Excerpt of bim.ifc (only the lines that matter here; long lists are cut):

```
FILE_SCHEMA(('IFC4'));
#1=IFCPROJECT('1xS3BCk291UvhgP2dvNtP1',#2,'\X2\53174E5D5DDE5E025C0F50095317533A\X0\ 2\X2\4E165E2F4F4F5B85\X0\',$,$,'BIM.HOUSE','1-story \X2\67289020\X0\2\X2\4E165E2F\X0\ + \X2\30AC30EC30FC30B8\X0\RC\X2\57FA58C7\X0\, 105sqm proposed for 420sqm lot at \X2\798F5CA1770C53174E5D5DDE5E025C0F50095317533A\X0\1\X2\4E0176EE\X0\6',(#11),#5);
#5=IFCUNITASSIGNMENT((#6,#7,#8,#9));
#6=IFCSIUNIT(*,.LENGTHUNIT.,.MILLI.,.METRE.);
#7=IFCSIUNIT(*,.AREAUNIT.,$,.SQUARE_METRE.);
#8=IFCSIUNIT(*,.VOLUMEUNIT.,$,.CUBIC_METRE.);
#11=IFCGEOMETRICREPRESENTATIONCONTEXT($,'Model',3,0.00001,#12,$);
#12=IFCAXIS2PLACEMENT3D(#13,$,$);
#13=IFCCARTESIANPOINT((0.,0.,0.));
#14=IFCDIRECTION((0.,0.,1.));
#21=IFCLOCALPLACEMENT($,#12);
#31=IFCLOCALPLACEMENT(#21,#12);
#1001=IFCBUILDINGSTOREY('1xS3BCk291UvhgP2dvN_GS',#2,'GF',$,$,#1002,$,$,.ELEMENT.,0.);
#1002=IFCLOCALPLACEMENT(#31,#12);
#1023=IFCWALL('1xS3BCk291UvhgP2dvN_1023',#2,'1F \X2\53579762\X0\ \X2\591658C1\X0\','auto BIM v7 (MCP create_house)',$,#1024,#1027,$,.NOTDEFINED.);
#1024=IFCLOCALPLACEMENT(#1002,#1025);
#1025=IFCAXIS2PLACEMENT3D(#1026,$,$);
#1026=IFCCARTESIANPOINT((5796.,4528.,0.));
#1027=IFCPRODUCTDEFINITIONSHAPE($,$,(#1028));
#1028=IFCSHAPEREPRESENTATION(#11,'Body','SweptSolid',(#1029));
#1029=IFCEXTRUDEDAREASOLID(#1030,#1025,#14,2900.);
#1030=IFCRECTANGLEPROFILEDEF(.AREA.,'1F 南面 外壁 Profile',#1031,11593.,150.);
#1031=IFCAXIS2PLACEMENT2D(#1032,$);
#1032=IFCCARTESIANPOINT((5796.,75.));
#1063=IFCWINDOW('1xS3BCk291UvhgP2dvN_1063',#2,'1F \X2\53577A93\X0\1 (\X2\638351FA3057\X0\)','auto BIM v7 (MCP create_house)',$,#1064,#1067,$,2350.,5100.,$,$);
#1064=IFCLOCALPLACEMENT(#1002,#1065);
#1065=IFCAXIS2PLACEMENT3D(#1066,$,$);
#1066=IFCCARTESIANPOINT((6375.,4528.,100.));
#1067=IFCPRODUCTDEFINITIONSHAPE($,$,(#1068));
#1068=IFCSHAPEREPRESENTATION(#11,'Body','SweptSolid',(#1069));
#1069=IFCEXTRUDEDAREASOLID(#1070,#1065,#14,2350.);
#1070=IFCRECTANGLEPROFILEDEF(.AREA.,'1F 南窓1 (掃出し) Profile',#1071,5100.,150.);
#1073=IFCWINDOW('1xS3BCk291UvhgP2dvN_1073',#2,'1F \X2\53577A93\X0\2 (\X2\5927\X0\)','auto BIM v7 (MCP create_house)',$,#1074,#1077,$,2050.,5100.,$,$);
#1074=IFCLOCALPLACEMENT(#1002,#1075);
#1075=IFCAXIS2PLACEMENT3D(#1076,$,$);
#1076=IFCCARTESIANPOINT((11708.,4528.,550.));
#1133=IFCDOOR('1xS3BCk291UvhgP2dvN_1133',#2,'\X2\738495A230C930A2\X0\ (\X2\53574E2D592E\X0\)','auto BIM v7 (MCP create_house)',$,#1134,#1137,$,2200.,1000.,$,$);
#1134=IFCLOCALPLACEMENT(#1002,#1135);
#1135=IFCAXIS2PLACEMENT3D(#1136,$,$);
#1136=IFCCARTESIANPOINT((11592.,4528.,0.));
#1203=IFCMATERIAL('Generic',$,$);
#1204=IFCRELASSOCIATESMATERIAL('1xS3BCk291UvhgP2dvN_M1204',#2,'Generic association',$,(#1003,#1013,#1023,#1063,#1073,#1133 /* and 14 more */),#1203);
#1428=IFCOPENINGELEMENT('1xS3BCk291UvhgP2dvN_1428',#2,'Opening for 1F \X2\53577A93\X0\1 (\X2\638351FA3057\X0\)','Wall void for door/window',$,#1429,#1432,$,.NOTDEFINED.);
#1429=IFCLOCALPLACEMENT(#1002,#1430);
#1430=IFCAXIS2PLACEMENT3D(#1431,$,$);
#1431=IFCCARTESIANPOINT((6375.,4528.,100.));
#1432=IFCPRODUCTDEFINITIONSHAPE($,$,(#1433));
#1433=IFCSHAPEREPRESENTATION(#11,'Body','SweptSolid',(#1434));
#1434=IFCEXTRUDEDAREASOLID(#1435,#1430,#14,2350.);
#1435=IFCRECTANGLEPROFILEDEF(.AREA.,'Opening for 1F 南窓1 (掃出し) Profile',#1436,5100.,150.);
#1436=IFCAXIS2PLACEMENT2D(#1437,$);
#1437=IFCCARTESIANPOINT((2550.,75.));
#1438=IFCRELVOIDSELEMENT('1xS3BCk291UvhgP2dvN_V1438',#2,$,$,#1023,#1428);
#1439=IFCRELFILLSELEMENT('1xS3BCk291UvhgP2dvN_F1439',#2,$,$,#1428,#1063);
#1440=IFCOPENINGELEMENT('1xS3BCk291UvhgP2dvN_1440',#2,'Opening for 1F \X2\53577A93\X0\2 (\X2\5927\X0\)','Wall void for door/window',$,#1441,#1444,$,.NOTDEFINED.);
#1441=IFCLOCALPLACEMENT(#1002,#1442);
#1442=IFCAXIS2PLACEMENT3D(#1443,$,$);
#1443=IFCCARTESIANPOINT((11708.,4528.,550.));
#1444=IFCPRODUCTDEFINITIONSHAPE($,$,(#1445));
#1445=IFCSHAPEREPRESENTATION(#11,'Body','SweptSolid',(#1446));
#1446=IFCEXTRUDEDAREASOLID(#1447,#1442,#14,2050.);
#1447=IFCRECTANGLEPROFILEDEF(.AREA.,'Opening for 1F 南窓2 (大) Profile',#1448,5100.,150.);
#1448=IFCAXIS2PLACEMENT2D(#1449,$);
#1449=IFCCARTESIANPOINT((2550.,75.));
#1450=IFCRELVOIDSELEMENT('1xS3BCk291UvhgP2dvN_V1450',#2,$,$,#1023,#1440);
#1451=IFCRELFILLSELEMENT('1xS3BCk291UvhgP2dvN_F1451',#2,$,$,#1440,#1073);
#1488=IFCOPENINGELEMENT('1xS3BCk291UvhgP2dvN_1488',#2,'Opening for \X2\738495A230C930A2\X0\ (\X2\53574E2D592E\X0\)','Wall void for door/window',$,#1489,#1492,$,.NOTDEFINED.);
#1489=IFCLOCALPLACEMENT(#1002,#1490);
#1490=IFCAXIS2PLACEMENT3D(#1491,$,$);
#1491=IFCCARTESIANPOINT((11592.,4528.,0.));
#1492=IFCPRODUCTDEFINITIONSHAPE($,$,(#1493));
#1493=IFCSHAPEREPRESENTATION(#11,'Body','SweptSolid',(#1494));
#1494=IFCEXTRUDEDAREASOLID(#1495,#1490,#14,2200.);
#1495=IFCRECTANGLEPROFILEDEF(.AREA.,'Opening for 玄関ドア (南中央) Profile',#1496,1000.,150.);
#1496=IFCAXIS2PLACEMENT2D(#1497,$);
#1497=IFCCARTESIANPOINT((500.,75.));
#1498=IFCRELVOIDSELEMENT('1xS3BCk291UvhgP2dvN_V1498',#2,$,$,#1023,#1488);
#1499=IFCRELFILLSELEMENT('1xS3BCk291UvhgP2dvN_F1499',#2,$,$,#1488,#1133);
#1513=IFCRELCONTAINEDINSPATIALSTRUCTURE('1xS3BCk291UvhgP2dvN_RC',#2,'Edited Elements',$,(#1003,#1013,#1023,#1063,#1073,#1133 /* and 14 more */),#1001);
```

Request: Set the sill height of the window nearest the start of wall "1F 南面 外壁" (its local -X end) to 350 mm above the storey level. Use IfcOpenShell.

```python
import numpy as np
import ifcopenshell
import ifcopenshell.api.geometry
import ifcopenshell.geom
import ifcopenshell.util.element
import ifcopenshell.util.placement
import ifcopenshell.util.shape
import ifcopenshell.util.unit

model = ifcopenshell.open("bim.ifc")
unit_scale = ifcopenshell.util.unit.calculate_unit_scale(model)

window = model.by_guid("1xS3BCk291UvhgP2dvN_1063")
opening = window.FillsVoids[0].RelatingOpeningElement
storey = ifcopenshell.util.element.get_container(window, ifc_class="IfcBuildingStorey")
level = ifcopenshell.util.placement.get_local_placement(storey.ObjectPlacement)[2, 3]

# The opening's origin need not be at the sill, so measure its lowest point.
shape = ifcopenshell.geom.create_shape(ifcopenshell.geom.settings(), opening)
bottom = ifcopenshell.util.shape.get_shape_bottom_elevation(shape, shape.geometry) / unit_scale
dz = level + 0.35 / unit_scale - bottom

shift = np.array([0.0, 0.0, dz])
# The window is not placed relative to its opening, so move both.
for product in (opening, window):
    matrix = ifcopenshell.util.placement.get_local_placement(product.ObjectPlacement)
    matrix[:3, 3] += shift
    ifcopenshell.api.geometry.edit_object_placement(model, product=product, matrix=matrix, is_si=False)

print(f"moved by {dz * unit_scale:+.3f} m")

model.write("bim_v2.ifc")
```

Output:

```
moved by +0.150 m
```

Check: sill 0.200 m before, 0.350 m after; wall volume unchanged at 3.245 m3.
